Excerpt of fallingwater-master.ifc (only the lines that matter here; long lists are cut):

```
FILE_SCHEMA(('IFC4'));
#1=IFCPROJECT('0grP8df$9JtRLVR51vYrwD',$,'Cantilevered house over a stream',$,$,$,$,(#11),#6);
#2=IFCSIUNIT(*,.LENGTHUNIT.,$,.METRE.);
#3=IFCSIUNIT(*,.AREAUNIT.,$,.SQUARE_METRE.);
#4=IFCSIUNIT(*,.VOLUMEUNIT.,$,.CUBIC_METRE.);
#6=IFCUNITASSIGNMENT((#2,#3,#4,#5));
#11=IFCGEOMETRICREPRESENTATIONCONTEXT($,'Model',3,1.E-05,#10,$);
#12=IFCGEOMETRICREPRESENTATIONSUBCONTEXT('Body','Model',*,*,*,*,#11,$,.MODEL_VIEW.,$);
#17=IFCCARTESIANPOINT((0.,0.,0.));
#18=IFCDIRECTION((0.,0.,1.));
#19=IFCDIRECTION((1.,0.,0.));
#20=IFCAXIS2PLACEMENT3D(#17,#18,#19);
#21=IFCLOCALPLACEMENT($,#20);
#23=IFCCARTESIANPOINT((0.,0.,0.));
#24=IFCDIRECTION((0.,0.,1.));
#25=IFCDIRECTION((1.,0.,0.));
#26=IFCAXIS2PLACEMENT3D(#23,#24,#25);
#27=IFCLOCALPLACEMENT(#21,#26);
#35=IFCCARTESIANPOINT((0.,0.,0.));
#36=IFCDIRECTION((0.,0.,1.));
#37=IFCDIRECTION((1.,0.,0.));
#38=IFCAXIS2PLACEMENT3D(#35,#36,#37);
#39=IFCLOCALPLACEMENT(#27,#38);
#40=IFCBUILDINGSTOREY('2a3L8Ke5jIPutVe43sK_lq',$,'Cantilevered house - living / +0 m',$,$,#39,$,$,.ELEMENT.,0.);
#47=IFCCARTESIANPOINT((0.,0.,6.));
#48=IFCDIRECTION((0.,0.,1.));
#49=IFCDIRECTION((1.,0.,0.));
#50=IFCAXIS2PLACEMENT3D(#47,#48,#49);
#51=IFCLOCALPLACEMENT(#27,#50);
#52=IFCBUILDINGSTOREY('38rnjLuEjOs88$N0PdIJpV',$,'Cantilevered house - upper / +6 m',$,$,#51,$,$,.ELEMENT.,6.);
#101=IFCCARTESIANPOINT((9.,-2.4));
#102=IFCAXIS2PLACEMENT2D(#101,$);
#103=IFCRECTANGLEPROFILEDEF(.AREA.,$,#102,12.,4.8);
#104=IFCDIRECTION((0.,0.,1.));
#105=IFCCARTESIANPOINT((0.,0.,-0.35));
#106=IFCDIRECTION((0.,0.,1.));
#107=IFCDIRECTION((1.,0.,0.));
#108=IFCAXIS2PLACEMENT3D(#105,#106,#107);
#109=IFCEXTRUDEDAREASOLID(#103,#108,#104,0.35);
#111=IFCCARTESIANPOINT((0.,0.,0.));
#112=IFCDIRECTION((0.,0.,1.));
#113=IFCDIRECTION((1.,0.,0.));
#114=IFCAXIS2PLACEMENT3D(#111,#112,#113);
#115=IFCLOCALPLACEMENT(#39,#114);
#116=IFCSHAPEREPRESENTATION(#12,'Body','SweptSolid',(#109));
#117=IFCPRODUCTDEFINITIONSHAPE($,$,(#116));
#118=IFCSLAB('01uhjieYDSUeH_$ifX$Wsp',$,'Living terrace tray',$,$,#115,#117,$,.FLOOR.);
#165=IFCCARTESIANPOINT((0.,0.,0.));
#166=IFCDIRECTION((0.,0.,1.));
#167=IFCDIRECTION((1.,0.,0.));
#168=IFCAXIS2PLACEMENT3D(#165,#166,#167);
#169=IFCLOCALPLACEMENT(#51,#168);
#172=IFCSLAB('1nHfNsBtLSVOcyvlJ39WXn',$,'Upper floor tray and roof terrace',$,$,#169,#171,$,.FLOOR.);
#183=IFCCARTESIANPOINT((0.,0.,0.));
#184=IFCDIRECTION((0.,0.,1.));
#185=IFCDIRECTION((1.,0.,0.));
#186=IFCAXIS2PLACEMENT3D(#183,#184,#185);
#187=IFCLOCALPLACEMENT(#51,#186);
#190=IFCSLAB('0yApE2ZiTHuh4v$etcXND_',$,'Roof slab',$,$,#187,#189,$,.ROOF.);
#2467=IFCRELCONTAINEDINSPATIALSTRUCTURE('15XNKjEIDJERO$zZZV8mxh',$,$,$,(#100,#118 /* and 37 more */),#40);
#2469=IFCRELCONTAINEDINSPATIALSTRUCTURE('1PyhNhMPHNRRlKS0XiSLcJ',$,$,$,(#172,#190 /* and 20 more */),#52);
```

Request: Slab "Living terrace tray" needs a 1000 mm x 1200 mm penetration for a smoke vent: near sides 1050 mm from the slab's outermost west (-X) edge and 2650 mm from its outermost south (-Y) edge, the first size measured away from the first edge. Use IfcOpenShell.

```python
import numpy as np
import ifcopenshell
import ifcopenshell.api.feature
import ifcopenshell.api.geometry
import ifcopenshell.api.root
import ifcopenshell.geom
import ifcopenshell.util.placement
import ifcopenshell.util.representation
import ifcopenshell.util.shape
import ifcopenshell.util.unit

model = ifcopenshell.open("fallingwater-master.ifc")
unit_scale = ifcopenshell.util.unit.calculate_unit_scale(model)
settings = ifcopenshell.geom.settings()


def volume(element):
    """Net volume in cubic metres, openings subtracted."""
    shape = ifcopenshell.geom.create_shape(settings, element)
    return ifcopenshell.util.shape.get_volume(shape.geometry)


slab = model.by_guid("01uhjieYDSUeH_$ifX$Wsp")
before = volume(slab)

# Extent in the slab's own axes, in metres. The edges named are its -X and -Y sides.
slab_shape = ifcopenshell.geom.create_shape(settings, slab)
vertices = ifcopenshell.util.shape.get_vertices(slab_shape.geometry)
x_min, y_min, bottom = vertices.min(axis=0)
top = vertices[:, 2].max()

opening = ifcopenshell.api.root.create_entity(model, ifc_class="IfcOpeningElement", name="Smoke vent opening", predefined_type="OPENING")
context = ifcopenshell.util.representation.get_context(model, "Model", "Body", "MODEL_VIEW")
width, depth = 1, 1.2
outline = [(0.0, 0.0), (width, 0.0), (width, depth), (0.0, depth), (0.0, 0.0)]
# Overshoot both faces by 50 mm so the cut is clean.
shape = ifcopenshell.api.geometry.add_slab_representation(
    model, context=context, depth=top - bottom + 0.1, polyline=outline
)
ifcopenshell.api.geometry.assign_representation(model, product=opening, representation=shape)

matrix = ifcopenshell.util.placement.get_local_placement(slab.ObjectPlacement)
matrix[:, 3] = matrix @ np.append(np.array([x_min + 1.05, y_min + 2.65, bottom - 0.05]) / unit_scale, 1.0)
ifcopenshell.api.geometry.edit_object_placement(model, product=opening, matrix=matrix, is_si=False)
ifcopenshell.api.feature.add_feature(model, feature=opening, element=slab)

after = volume(slab)

print(f"slab volume {before:.3f} -> {after:.3f} m3")

model.write("fallingwater-master_rev.ifc")
```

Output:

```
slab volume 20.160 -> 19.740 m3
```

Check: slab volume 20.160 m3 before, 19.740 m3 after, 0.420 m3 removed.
